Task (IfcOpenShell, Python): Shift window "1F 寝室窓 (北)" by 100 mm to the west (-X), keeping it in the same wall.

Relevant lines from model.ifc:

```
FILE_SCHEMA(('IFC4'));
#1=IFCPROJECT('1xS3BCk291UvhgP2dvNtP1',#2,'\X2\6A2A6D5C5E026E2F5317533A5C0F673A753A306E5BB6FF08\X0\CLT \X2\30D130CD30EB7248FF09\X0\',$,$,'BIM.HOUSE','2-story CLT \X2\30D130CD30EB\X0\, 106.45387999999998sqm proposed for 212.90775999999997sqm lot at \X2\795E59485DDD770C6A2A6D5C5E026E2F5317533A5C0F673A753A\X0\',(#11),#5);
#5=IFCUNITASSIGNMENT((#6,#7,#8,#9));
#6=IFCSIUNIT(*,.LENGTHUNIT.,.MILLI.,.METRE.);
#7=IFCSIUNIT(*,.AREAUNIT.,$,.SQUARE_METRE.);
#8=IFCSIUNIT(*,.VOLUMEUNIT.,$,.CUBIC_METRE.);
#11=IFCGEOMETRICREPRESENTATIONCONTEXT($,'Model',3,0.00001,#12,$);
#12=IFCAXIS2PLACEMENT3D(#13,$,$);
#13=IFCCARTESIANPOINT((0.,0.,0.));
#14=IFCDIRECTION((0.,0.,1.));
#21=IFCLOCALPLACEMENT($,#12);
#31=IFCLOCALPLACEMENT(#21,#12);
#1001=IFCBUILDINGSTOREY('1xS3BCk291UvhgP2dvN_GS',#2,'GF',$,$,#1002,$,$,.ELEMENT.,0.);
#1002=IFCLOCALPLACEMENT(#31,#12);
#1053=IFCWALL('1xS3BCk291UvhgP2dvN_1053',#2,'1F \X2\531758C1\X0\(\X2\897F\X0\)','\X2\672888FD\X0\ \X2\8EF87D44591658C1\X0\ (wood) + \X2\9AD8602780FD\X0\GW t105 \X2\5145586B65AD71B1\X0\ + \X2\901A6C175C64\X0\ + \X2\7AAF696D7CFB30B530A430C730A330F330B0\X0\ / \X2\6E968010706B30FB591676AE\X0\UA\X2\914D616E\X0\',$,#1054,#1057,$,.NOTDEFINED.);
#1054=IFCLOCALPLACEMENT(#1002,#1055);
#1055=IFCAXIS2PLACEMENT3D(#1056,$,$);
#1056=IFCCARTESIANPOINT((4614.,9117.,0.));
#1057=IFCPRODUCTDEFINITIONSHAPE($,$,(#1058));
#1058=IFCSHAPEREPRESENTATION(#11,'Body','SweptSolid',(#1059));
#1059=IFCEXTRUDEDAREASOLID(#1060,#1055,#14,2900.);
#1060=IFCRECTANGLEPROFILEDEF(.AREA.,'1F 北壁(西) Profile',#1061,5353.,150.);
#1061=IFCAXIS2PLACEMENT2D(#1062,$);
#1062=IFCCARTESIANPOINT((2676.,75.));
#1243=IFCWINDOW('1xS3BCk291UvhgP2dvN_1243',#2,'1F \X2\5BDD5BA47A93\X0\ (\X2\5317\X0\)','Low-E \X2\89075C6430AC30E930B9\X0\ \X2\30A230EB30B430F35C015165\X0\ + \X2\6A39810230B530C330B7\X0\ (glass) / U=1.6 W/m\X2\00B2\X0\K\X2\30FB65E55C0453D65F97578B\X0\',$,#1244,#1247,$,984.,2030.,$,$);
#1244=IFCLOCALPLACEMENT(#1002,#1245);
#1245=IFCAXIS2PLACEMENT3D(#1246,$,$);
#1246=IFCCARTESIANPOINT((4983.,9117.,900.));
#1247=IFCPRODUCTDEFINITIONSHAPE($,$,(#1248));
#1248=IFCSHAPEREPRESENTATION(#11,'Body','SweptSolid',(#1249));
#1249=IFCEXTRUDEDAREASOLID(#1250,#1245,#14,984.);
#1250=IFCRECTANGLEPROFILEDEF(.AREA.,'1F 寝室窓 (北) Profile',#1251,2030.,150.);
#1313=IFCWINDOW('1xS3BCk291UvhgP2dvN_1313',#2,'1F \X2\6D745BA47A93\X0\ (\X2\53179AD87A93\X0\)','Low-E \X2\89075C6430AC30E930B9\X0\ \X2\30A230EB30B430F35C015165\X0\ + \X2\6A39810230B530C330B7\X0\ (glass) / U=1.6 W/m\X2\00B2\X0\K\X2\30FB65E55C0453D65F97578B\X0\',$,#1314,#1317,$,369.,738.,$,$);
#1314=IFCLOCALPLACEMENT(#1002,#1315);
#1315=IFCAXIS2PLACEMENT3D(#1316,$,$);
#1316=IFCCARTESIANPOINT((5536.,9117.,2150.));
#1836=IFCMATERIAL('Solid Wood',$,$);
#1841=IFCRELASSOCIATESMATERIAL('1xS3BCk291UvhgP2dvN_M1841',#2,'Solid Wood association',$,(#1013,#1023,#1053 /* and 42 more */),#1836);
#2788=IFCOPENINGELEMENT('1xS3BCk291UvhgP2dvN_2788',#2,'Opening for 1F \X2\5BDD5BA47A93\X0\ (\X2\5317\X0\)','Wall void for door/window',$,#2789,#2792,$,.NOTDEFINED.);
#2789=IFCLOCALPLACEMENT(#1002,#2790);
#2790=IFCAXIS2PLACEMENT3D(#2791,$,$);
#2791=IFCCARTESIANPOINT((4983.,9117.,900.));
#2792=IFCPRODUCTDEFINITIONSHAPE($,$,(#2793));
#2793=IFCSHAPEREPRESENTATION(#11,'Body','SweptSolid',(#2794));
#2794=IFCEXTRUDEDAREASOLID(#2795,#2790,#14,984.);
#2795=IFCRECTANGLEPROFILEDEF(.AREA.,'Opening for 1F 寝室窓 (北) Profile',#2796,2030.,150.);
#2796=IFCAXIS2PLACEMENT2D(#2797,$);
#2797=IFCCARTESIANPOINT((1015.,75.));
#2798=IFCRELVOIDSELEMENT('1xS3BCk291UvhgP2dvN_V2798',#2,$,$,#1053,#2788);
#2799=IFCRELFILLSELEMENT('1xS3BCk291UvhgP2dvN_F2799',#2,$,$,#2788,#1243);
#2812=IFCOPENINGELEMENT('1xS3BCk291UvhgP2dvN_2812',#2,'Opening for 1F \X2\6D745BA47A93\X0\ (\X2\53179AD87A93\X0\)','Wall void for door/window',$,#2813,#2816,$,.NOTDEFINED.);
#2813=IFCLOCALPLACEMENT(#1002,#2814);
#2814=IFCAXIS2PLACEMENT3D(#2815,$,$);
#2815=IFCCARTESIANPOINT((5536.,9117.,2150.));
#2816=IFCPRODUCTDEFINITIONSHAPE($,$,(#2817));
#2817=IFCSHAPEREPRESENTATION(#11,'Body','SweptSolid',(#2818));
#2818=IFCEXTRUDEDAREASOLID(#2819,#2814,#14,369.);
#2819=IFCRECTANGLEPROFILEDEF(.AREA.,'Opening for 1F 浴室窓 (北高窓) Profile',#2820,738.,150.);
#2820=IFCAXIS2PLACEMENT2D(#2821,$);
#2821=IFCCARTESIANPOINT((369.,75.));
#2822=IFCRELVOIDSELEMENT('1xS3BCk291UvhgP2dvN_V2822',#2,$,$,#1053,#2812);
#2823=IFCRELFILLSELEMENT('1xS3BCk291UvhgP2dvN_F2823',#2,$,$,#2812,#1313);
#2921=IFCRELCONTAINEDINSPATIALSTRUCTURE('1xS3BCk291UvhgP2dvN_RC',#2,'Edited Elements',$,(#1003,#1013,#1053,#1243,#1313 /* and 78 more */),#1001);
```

```python
import ifcopenshell
import ifcopenshell.api.geometry
import ifcopenshell.util.placement
import ifcopenshell.util.unit

model = ifcopenshell.open("model.ifc")
unit_scale = ifcopenshell.util.unit.calculate_unit_scale(model)

window = model.by_id(1243)
opening = window.FillsVoids[0].RelatingOpeningElement
wall = opening.VoidsElements[0].RelatingBuildingElement

wall_matrix = ifcopenshell.util.placement.get_local_placement(wall.ObjectPlacement)
shift = wall_matrix[:3, 0] * -0.1 / unit_scale
before = ifcopenshell.util.placement.get_local_placement(window.ObjectPlacement)[:3, 3].copy()

# The window is not placed relative to its opening, so move both.
for product in (opening, window):
    matrix = ifcopenshell.util.placement.get_local_placement(product.ObjectPlacement)
    matrix[:3, 3] += shift
    ifcopenshell.api.geometry.edit_object_placement(model, product=product, matrix=matrix, is_si=False)

after = ifcopenshell.util.placement.get_local_placement(window.ObjectPlacement)[:3, 3]
print("window moved by", (after - before).round(3) + 0.0)

model.write("model_updated.ifc")
```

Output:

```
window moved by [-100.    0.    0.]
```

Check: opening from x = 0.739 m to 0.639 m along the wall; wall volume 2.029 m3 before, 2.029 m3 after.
